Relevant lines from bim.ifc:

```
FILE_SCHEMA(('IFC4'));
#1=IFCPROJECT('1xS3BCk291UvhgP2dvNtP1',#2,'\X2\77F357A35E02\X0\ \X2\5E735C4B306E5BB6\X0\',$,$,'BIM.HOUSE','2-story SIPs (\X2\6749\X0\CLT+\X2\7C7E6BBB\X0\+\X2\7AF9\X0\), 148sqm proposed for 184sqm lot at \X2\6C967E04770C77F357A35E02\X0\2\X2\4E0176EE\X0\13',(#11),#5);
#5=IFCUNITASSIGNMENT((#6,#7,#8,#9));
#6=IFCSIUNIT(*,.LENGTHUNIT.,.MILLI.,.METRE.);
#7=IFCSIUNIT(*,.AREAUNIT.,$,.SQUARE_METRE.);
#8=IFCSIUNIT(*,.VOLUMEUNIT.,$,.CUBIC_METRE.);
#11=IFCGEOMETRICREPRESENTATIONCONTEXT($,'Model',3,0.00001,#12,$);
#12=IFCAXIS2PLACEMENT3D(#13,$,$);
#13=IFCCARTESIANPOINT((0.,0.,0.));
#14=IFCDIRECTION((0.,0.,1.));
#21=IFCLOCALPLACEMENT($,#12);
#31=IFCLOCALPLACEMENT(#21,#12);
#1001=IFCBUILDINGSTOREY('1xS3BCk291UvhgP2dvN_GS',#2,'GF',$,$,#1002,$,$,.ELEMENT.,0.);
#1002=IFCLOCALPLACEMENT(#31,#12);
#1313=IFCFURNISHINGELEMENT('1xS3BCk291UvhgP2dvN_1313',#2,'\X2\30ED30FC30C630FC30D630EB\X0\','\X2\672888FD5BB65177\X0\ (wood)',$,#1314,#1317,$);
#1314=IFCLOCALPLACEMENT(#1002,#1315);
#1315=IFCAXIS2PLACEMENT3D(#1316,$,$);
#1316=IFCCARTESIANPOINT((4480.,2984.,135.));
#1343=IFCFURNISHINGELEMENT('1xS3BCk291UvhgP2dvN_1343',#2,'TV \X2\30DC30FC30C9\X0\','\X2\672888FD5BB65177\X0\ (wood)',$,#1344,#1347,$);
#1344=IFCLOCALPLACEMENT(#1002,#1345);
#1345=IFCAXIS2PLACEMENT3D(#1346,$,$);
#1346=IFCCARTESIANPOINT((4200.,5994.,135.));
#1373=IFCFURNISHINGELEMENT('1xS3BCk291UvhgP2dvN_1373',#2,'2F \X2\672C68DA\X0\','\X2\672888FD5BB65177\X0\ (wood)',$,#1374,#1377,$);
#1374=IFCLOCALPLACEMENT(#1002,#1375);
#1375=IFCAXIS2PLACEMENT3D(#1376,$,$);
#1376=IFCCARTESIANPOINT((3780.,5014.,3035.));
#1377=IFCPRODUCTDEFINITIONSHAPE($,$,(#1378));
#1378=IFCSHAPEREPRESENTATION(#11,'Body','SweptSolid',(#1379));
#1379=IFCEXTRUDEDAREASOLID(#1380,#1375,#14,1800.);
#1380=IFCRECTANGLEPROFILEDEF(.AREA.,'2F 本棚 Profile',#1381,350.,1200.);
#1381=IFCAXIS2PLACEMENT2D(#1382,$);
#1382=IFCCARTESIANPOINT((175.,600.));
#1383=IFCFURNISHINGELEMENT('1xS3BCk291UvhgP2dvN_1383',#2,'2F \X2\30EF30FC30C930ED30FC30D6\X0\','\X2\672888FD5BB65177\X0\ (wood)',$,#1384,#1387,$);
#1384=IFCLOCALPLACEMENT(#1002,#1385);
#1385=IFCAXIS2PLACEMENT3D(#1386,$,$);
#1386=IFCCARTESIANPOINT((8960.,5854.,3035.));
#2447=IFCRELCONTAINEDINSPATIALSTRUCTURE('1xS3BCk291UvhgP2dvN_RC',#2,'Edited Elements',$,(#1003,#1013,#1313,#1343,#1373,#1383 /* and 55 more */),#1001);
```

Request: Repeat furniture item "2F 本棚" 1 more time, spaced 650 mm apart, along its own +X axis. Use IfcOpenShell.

```python
import ifcopenshell
import ifcopenshell.api.geometry
import ifcopenshell.api.root
import ifcopenshell.util.element
import ifcopenshell.util.placement
import ifcopenshell.util.unit

model = ifcopenshell.open("bim.ifc")
unit_scale = ifcopenshell.util.unit.calculate_unit_scale(model)


def reuse_history(source, copy):
    """copy_class also copies each property set's owner history, people and application; keep the originals."""
    for rel in copy.IsDefinedBy:
        if rel.is_a("IfcRelDefinesByProperties") and (history := rel.RelatingPropertyDefinition.OwnerHistory):
            rel.RelatingPropertyDefinition.OwnerHistory = source.OwnerHistory
            ifcopenshell.util.element.remove_deep2(model, history)


source = model.by_id(1373)
base = ifcopenshell.util.placement.get_local_placement(source.ObjectPlacement)
step = base[:3, 0] * 0.65 / unit_scale

for i in range(1, 2):
    copy = ifcopenshell.api.root.copy_class(model, product=source)
    copy.Representation = ifcopenshell.util.element.copy_deep(
        model, source.Representation, exclude=["IfcGeometricRepresentationContext", "IfcRepresentationMap"]
    )
    reuse_history(source, copy)
    matrix = base.copy()
    matrix[:3, 3] += i * step
    print("added at", matrix[:3, 3].round(3) + 0.0)
    ifcopenshell.api.geometry.edit_object_placement(model, product=copy, matrix=matrix, is_si=False)

model.write("bim_edited.ifc")
```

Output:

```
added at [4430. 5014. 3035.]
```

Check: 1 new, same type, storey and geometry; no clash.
